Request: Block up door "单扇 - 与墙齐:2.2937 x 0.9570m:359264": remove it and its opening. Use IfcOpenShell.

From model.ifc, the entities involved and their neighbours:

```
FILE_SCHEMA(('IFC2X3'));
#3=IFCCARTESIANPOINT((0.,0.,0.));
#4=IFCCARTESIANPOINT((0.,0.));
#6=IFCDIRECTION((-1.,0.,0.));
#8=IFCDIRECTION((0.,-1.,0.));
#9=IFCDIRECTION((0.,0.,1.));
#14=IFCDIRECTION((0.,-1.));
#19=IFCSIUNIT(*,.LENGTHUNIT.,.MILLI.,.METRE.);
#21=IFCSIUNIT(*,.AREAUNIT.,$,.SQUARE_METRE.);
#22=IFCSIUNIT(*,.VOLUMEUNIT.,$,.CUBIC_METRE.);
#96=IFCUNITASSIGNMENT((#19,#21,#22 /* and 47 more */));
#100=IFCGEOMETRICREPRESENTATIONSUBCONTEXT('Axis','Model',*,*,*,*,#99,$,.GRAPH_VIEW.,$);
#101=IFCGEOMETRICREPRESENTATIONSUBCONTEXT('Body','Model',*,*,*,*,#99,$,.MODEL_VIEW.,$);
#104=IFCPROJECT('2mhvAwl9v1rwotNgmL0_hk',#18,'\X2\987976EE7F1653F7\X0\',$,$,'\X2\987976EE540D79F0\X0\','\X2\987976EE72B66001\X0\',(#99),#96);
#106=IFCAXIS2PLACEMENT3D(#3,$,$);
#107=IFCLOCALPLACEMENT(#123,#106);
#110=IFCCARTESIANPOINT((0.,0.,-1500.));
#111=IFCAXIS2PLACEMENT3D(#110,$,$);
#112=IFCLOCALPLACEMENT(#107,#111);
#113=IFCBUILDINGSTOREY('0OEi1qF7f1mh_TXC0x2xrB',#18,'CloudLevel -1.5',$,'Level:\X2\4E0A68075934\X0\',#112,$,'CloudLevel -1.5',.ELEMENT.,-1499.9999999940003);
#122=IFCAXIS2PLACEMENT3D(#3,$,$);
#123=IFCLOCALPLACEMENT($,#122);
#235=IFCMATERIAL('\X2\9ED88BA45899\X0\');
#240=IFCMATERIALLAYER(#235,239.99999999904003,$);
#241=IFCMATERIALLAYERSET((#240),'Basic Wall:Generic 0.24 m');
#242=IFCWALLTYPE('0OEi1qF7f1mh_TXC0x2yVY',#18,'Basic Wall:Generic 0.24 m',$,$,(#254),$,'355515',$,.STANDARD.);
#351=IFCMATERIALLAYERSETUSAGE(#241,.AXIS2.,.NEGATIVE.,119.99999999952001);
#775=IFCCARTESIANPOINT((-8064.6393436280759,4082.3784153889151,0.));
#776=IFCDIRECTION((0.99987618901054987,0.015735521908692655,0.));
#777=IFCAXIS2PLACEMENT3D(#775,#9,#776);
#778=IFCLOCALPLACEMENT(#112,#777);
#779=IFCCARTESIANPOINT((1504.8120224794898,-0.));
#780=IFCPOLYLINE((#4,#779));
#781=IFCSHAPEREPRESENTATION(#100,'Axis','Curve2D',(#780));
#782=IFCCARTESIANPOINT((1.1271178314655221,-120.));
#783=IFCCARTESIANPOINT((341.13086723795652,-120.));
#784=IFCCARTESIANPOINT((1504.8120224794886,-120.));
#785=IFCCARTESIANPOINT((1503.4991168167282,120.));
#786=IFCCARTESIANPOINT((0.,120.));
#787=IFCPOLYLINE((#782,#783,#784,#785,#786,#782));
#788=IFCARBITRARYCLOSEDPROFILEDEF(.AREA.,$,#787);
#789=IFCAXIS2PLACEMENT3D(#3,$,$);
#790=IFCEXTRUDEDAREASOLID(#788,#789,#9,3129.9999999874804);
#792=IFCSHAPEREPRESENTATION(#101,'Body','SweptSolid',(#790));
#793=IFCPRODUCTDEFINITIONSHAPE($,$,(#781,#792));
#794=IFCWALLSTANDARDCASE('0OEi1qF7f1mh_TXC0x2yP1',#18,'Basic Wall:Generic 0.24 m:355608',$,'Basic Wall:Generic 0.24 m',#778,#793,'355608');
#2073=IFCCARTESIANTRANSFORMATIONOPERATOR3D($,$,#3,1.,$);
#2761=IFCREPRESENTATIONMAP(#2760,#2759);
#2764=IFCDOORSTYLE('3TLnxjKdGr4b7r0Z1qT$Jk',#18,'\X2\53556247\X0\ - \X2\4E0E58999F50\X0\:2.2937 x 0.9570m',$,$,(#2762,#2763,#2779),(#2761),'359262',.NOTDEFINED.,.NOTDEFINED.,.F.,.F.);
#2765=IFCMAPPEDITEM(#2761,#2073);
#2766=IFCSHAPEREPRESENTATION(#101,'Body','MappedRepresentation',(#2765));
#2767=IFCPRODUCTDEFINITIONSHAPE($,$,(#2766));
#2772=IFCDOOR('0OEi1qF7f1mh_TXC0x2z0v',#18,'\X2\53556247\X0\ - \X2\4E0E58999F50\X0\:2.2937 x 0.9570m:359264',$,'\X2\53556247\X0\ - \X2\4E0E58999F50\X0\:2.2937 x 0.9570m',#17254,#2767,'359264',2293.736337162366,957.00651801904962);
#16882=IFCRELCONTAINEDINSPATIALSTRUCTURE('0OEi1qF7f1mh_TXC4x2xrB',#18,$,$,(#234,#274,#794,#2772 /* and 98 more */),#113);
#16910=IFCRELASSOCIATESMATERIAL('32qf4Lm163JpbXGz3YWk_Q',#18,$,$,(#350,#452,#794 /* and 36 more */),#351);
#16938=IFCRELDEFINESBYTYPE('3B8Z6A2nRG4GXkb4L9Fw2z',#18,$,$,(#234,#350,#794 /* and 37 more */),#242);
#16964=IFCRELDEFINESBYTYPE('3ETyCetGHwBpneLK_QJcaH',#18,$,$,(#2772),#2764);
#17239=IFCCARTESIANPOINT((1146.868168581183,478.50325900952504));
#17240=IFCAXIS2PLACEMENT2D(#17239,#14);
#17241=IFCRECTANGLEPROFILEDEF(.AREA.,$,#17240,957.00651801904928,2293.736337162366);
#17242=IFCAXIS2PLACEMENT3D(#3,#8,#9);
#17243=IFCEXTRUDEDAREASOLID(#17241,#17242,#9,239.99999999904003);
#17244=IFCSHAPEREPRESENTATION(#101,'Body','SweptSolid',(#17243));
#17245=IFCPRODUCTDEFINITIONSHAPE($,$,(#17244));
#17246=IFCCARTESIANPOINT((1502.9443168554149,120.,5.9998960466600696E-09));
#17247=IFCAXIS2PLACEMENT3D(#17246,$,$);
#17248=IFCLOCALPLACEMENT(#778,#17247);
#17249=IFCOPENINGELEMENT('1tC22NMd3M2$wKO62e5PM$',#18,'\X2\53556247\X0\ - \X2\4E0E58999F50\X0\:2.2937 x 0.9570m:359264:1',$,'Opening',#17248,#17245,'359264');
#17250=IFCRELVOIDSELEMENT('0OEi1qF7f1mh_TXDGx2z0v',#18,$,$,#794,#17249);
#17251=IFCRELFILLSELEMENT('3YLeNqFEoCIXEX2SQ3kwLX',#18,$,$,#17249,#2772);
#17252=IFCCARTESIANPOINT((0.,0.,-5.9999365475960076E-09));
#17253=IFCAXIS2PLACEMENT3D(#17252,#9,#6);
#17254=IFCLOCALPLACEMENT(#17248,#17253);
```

```python
import ifcopenshell
import ifcopenshell.api.feature
import ifcopenshell.api.root
import ifcopenshell.geom
import ifcopenshell.util.shape

model = ifcopenshell.open("model.ifc")
settings = ifcopenshell.geom.settings()


def volume(element):
    """Net volume in cubic metres, openings subtracted."""
    shape = ifcopenshell.geom.create_shape(settings, element)
    return ifcopenshell.util.shape.get_volume(shape.geometry)


door = model.by_guid("0OEi1qF7f1mh_TXC0x2z0v")
opening = door.FillsVoids[0].RelatingOpeningElement
wall = opening.VoidsElements[0].RelatingBuildingElement
before = volume(wall)

ifcopenshell.api.root.remove_product(model, product=door)
ifcopenshell.api.feature.remove_feature(model, feature=opening)

after = volume(wall)

print(f"wall volume {before:.3f} -> {after:.3f} m3")

model.write("model_edited.ifc")
```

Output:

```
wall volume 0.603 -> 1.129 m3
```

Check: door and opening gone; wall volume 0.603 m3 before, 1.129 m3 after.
